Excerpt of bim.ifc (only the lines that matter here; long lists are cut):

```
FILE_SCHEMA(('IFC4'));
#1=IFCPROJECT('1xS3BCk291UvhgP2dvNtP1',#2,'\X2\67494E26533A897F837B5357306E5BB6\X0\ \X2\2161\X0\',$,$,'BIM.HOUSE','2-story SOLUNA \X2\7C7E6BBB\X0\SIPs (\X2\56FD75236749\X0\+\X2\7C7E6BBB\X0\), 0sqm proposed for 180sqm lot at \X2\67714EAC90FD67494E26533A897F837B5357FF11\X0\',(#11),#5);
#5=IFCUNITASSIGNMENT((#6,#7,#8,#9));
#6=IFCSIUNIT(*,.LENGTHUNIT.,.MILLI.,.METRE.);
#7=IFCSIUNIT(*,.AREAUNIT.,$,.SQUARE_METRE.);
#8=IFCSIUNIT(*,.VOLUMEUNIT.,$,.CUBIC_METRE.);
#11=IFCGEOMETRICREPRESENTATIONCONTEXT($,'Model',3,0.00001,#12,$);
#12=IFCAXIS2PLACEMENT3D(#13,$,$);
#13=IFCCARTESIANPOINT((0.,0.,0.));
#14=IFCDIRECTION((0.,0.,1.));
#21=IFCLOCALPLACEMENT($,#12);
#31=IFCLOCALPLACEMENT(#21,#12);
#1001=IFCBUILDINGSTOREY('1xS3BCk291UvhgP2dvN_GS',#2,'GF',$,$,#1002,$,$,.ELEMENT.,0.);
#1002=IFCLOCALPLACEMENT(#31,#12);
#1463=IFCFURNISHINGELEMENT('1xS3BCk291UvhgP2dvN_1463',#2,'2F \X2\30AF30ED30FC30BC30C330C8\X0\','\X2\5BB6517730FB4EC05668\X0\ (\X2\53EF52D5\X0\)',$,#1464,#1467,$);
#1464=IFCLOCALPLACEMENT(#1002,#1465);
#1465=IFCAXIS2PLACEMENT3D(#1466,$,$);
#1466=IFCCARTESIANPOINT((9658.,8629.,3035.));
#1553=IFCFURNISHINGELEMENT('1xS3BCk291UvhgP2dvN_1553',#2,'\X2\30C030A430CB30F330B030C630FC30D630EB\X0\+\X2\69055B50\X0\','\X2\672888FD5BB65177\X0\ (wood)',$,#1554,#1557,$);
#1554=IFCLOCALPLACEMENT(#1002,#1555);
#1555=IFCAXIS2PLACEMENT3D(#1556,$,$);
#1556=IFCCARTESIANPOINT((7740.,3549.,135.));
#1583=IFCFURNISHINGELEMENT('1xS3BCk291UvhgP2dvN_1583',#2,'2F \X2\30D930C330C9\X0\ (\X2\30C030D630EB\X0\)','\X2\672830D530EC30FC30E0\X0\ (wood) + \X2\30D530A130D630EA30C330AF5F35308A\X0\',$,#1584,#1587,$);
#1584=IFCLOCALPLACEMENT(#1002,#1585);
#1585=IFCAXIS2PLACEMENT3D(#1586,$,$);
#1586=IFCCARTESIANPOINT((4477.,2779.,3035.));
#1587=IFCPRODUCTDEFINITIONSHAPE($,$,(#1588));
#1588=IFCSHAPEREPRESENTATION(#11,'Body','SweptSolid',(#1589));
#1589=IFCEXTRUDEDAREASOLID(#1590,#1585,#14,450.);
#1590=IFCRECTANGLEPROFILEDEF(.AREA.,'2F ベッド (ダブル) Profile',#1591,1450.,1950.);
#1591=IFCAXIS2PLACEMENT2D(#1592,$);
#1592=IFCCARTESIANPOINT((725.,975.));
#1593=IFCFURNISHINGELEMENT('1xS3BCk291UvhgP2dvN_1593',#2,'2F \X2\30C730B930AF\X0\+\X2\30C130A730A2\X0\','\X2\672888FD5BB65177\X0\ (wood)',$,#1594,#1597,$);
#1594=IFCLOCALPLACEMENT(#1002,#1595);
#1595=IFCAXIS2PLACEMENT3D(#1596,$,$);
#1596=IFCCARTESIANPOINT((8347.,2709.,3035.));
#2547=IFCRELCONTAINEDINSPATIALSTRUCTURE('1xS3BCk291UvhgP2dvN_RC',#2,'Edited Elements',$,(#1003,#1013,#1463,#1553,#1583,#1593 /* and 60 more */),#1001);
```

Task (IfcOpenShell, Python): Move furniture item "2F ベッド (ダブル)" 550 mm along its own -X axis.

```python
import ifcopenshell
import ifcopenshell.api.geometry
import ifcopenshell.util.placement

model = ifcopenshell.open("bim.ifc")

item = model.by_guid("1xS3BCk291UvhgP2dvN_1583")
matrix = ifcopenshell.util.placement.get_local_placement(item.ObjectPlacement)
matrix[:3, 3] -= matrix[:3, 0] * 550.0
ifcopenshell.api.geometry.edit_object_placement(model, product=item, matrix=matrix, is_si=False)

print(ifcopenshell.util.placement.get_local_placement(item.ObjectPlacement).round(3) + 0.0)

model.write("bim_edited.ifc")
```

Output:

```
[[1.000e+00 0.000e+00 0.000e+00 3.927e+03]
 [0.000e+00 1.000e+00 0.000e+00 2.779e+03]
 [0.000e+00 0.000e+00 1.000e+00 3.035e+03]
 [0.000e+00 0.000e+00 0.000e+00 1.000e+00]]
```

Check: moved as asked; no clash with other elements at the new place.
